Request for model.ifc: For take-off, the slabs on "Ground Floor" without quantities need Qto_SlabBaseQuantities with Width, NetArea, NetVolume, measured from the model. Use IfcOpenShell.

First a look at what the model holds.

```python
import ifcopenshell
import ifcopenshell.util.element
import ifcopenshell.util.unit

model = ifcopenshell.open("model.ifc")
print(model.schema)
for unit_type in ("LENGTHUNIT", "AREAUNIT", "VOLUMEUNIT"):
    print(unit_type, ifcopenshell.util.unit.calculate_unit_scale(model, unit_type))
storey = next(s for s in model.by_type("IfcBuildingStorey") if s.Name == "Ground Floor")
slabs = [e for e in ifcopenshell.util.element.get_decomposition(storey) if e.is_a("IfcSlab")]
for e in sorted(slabs, key=lambda e: e.id()):
    print(e.id(), e.is_a(), e.Name, list(ifcopenshell.util.element.get_psets(e, qtos_only=True)), sep=" | ")
```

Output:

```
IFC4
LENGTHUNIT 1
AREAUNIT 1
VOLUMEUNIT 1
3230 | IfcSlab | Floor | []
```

```python
import ifcopenshell
import ifcopenshell.api.pset
import ifcopenshell.geom
import ifcopenshell.util.element
import ifcopenshell.util.shape
import ifcopenshell.util.unit

model = ifcopenshell.open("model.ifc")
unit_scale = ifcopenshell.util.unit.calculate_unit_scale(model)
area_scale = ifcopenshell.util.unit.calculate_unit_scale(model, "AREAUNIT")
volume_scale = ifcopenshell.util.unit.calculate_unit_scale(model, "VOLUMEUNIT")
settings = ifcopenshell.geom.settings()

storey = next(s for s in model.by_type("IfcBuildingStorey") if s.Name == "Ground Floor")
slabs = [e for e in ifcopenshell.util.element.get_decomposition(storey) if e.is_a("IfcSlab")]

for e in sorted(slabs, key=lambda e: e.id()):
    if ifcopenshell.util.element.get_psets(e, qtos_only=True, should_inherit=False):
        continue
    # Geometry comes back in metres, in the element's own axes.
    shape = ifcopenshell.geom.create_shape(settings, e)
    values = {
        "Width": ifcopenshell.util.shape.get_z(shape.geometry) / unit_scale,
        "NetArea": ifcopenshell.util.shape.get_footprint_area(shape.geometry) / area_scale,
        "NetVolume": ifcopenshell.util.shape.get_volume(shape.geometry) / volume_scale,
    }
    qto = ifcopenshell.api.pset.add_qto(model, product=e, name="Qto_SlabBaseQuantities")
    ifcopenshell.api.pset.edit_qto(model, qto=qto, properties=values)
    print(e.id(), {k: round(v, 3) for k, v in values.items()})

model.write("model_v2.ifc")
```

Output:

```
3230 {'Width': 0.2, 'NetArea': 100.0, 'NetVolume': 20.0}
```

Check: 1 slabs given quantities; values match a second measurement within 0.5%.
